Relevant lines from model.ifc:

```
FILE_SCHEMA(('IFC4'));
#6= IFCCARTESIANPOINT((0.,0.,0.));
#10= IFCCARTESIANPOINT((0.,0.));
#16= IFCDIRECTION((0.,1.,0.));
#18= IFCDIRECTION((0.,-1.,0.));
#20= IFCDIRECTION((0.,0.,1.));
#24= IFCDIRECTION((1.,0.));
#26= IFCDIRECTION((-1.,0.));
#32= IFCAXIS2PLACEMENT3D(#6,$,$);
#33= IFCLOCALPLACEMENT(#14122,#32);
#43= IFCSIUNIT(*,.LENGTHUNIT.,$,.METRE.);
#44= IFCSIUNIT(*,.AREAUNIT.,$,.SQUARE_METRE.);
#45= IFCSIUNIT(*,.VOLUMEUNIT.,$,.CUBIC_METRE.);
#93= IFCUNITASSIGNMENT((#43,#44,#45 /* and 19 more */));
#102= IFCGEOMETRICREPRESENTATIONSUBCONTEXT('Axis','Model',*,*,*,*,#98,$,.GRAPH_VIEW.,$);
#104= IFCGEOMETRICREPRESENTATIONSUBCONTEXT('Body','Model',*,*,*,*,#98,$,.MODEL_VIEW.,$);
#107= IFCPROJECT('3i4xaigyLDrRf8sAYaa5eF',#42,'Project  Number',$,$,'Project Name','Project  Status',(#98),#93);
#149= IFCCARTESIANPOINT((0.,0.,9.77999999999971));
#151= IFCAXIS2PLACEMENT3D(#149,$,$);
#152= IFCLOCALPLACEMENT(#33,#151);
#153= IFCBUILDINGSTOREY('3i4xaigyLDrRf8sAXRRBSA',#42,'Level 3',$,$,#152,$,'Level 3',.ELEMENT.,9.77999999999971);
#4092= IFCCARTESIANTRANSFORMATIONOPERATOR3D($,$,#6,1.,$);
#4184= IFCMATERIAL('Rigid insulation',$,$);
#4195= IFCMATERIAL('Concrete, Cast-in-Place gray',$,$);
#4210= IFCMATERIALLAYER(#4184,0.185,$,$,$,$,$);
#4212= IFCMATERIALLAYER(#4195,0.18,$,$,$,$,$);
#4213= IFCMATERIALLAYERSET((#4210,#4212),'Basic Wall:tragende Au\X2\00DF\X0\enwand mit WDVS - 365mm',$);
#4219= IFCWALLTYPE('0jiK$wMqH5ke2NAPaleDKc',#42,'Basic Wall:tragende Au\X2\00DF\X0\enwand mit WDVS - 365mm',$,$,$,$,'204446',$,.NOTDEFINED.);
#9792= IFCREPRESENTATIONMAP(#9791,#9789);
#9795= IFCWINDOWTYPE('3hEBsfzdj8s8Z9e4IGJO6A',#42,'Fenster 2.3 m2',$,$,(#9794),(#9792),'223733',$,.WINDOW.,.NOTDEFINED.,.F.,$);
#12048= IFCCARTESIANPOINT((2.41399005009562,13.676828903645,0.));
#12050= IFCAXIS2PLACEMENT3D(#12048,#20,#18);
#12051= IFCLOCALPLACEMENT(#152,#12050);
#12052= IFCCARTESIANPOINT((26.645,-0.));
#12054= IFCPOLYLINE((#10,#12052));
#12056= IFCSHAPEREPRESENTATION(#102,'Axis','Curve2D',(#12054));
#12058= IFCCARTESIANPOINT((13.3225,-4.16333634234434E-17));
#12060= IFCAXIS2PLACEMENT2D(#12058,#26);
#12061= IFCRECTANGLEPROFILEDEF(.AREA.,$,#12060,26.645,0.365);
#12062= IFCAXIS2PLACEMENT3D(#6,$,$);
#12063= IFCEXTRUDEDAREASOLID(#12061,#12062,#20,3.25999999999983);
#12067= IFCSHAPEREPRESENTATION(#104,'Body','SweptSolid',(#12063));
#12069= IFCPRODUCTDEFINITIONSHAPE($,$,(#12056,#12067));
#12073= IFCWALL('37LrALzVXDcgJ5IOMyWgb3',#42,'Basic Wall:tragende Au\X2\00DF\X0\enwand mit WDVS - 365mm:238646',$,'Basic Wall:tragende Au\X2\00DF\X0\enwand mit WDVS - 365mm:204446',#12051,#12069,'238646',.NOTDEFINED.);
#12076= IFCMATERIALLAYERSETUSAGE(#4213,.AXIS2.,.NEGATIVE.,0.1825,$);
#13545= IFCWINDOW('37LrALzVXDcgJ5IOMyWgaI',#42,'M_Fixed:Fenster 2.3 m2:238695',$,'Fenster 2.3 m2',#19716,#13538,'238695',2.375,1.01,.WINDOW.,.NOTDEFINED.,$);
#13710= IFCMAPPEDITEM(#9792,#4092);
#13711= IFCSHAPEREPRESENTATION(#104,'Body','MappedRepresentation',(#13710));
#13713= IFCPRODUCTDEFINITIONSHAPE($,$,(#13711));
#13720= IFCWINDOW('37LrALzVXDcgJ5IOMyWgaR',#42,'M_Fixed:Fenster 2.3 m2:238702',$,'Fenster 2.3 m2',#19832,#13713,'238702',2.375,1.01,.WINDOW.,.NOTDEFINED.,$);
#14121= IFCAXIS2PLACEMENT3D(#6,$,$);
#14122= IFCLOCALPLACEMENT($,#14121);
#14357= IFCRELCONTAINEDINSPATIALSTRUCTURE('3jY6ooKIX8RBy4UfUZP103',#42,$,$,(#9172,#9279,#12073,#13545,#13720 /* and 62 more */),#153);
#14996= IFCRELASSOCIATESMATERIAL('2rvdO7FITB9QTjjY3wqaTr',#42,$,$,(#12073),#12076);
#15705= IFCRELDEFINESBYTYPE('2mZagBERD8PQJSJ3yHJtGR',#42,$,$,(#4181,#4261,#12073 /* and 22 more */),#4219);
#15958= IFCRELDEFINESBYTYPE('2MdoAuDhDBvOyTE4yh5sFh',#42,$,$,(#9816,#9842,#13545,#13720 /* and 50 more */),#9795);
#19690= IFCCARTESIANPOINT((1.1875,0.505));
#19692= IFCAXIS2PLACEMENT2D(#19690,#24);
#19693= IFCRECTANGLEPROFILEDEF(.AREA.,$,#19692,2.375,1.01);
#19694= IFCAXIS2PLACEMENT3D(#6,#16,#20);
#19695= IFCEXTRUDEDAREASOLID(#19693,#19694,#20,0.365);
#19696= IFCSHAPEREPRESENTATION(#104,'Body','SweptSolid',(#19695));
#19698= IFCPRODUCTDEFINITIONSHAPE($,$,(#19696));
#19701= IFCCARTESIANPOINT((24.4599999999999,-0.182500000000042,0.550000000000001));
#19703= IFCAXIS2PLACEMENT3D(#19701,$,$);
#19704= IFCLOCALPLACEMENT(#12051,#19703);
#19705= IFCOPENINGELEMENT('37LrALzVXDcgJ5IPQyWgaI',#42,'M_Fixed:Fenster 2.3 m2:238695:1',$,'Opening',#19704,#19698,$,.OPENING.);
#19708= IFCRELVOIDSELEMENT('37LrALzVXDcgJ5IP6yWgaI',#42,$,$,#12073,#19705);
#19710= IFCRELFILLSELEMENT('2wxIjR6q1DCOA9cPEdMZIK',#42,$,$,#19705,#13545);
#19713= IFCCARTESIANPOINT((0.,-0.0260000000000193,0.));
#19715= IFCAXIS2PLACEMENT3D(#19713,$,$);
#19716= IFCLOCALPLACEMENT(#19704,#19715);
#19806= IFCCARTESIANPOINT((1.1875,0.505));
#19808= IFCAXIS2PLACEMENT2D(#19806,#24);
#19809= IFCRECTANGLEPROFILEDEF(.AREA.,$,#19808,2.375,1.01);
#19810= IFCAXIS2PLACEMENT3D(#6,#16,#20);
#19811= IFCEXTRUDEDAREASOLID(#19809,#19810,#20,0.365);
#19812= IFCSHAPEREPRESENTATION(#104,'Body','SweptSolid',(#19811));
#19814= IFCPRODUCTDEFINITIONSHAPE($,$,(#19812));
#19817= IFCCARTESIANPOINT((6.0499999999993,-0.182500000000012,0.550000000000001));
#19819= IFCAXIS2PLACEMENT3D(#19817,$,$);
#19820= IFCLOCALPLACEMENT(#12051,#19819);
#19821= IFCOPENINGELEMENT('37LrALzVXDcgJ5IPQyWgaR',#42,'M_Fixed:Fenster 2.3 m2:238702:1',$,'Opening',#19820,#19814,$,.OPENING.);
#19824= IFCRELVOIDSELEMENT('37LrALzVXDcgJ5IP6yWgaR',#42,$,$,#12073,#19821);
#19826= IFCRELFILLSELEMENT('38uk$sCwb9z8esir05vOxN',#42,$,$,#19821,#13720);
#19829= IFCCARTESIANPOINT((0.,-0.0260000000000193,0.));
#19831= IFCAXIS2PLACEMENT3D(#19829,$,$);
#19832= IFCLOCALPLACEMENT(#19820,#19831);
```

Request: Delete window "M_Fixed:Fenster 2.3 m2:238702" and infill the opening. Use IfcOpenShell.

```python
import ifcopenshell
import ifcopenshell.api.feature
import ifcopenshell.api.root
import ifcopenshell.geom
import ifcopenshell.util.shape

model = ifcopenshell.open("model.ifc")
settings = ifcopenshell.geom.settings()


def volume(element):
    """Net volume in cubic metres, openings subtracted."""
    shape = ifcopenshell.geom.create_shape(settings, element)
    return ifcopenshell.util.shape.get_volume(shape.geometry)


window = model.by_id(13720)
opening = window.FillsVoids[0].RelatingOpeningElement
wall = opening.VoidsElements[0].RelatingBuildingElement
before = volume(wall)

ifcopenshell.api.root.remove_product(model, product=window)
ifcopenshell.api.feature.remove_feature(model, feature=opening)

after = volume(wall)

print(f"wall volume {before:.3f} -> {after:.3f} m3")

model.write("model_edited.ifc")
```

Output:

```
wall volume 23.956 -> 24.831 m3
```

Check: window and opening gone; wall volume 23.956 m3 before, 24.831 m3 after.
